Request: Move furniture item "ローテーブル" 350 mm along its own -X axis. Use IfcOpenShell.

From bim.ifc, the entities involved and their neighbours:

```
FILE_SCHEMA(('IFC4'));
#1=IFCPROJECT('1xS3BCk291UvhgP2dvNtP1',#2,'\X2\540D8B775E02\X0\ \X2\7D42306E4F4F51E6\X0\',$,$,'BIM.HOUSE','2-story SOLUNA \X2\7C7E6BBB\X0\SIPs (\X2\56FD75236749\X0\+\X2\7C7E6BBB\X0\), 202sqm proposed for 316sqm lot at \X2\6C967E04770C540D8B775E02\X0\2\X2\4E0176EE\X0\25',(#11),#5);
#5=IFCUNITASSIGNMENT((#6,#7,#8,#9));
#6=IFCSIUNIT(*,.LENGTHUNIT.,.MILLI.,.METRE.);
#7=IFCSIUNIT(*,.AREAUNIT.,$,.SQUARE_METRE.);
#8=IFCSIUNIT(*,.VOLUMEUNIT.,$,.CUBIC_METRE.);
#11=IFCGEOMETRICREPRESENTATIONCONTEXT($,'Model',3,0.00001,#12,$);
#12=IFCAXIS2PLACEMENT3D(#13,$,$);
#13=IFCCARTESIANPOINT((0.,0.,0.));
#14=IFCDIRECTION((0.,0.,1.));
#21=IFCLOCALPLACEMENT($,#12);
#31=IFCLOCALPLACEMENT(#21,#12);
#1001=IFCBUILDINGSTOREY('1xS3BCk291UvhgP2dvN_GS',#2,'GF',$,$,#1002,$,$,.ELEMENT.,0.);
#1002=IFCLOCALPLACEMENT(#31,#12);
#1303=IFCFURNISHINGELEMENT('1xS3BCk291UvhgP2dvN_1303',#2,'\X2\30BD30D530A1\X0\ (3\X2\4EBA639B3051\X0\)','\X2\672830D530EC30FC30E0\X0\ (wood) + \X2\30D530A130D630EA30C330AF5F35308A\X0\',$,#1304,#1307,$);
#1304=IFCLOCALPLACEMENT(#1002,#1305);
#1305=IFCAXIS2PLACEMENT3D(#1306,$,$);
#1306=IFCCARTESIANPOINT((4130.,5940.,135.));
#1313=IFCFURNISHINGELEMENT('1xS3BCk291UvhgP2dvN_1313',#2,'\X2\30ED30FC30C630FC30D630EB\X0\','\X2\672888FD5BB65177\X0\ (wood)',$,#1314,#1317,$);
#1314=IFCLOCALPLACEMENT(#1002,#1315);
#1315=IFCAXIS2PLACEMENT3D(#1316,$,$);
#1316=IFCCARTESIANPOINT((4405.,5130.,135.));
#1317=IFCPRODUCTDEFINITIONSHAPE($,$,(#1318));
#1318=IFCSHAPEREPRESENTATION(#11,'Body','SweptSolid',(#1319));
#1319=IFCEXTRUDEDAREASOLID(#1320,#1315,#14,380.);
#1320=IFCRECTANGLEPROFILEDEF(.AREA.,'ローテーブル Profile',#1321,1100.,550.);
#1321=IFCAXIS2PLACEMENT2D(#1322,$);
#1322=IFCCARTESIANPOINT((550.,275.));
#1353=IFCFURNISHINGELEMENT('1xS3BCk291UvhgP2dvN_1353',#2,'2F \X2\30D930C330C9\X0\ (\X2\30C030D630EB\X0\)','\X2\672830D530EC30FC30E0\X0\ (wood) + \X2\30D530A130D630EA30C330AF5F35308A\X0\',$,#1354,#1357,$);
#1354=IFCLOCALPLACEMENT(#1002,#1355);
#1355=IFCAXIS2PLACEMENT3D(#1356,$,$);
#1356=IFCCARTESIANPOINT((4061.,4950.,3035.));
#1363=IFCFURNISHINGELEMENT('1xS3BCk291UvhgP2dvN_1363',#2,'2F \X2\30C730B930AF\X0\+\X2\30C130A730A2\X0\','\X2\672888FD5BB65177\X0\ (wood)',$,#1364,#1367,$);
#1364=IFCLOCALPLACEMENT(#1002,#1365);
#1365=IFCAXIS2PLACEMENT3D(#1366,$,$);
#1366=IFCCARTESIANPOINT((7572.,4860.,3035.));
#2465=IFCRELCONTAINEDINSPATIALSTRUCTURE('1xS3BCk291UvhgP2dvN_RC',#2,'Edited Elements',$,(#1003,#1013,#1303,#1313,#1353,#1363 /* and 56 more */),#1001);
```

```python
import ifcopenshell
import ifcopenshell.api.geometry
import ifcopenshell.util.placement
import ifcopenshell.util.unit

model = ifcopenshell.open("bim.ifc")
unit_scale = ifcopenshell.util.unit.calculate_unit_scale(model)

item = model.by_guid("1xS3BCk291UvhgP2dvN_1313")
matrix = ifcopenshell.util.placement.get_local_placement(item.ObjectPlacement)
matrix[:3, 3] -= matrix[:3, 0] * 0.35 / unit_scale
ifcopenshell.api.geometry.edit_object_placement(model, product=item, matrix=matrix, is_si=False)

print(ifcopenshell.util.placement.get_local_placement(item.ObjectPlacement).round(3) + 0.0)

model.write("bim_updated.ifc")
```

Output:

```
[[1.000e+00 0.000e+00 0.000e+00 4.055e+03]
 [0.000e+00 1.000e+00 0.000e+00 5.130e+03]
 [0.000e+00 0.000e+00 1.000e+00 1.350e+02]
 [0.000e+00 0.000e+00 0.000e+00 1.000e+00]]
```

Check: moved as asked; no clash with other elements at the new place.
